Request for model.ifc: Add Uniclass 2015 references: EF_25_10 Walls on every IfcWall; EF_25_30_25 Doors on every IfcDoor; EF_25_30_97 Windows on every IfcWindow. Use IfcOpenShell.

First a look at what the model holds.

```python
import ifcopenshell

model = ifcopenshell.open("model.ifc")
print(model.schema)
print("classifications:", [c.Name for c in model.by_type("IfcClassification")])
for ifc_class in ("IfcDoor", "IfcRoof", "IfcStair", "IfcWall", "IfcWindow"):
    print(ifc_class, len(model.by_type(ifc_class)))
```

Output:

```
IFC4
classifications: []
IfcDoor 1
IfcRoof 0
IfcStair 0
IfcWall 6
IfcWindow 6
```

```python
import ifcopenshell
import ifcopenshell.api.classification

model = ifcopenshell.open("model.ifc")

system = ifcopenshell.api.classification.add_classification(model, classification="Uniclass 2015")

codes = {
    "IfcWall": ("EF_25_10", "Walls"),
    "IfcDoor": ("EF_25_30_25", "Doors"),
    "IfcWindow": ("EF_25_30_97", "Windows"),
}
for ifc_class, (code, name) in codes.items():
    products = model.by_type(ifc_class)
    ifcopenshell.api.classification.add_reference(
        model, products=products, classification=system, identification=code, name=name
    )
    print(code, len(products))

model.write("model_rev.ifc")
```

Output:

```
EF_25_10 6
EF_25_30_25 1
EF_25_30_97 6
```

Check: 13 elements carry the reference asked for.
